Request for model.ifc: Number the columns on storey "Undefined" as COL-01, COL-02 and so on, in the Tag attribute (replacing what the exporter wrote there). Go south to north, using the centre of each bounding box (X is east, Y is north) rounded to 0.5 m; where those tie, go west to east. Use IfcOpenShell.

First a look at what the model holds.

```python
import ifcopenshell
import ifcopenshell.util.element
import ifcopenshell.util.placement

model = ifcopenshell.open("model.ifc")
print(model.schema)
storey = next(s for s in model.by_type("IfcBuildingStorey") if s.Name == "Undefined")
columns = [e for e in ifcopenshell.util.element.get_decomposition(storey) if e.is_a("IfcColumn")]
for e in sorted(columns, key=lambda e: e.id()):
    origin = ifcopenshell.util.placement.get_local_placement(e.ObjectPlacement)[:3, 3]
    print(e.id(), e.Tag, e.Name, origin.round(2) + 0.0, sep=" | ")
```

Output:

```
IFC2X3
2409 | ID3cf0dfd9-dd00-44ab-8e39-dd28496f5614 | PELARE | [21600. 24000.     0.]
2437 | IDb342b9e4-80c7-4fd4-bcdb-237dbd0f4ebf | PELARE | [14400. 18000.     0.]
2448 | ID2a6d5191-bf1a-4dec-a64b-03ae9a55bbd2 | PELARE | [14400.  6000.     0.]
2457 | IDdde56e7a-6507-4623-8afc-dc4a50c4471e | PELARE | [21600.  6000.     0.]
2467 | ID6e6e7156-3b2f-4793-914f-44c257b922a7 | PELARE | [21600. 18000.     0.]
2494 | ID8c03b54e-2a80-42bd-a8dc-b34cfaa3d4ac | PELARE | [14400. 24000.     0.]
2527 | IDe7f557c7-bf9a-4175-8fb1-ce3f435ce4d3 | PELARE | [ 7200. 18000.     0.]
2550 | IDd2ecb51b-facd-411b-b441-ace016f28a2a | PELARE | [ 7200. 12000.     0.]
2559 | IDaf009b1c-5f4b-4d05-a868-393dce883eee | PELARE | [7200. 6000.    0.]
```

```python
import ifcopenshell
import ifcopenshell.geom
import ifcopenshell.util.element
import ifcopenshell.util.shape

model = ifcopenshell.open("model.ifc")
settings = ifcopenshell.geom.settings()
settings.set("use-world-coords", True)


def centre(element):
    shape = ifcopenshell.geom.create_shape(settings, element)
    return ifcopenshell.util.shape.get_bbox_centroid(shape.geometry)


storey = next(s for s in model.by_type("IfcBuildingStorey") if s.Name == "Undefined")
columns = [e for e in ifcopenshell.util.element.get_decomposition(storey) if e.is_a("IfcColumn")]

# Insertion points can sit at a corner or the storey origin, so sort by the geometry (in metres).
centres = {e: centre(e) for e in columns}
columns.sort(key=lambda e: (round(centres[e][1] / 0.5), centres[e][0]))

for i, e in enumerate(columns, start=1):
    number = f"COL-{i:02d}"
    e.Tag = number
    print(e.id(), number)

model.write("model_edited.ifc")
```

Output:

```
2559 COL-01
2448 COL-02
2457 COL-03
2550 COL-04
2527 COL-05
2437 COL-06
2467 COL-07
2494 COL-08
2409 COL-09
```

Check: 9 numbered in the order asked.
